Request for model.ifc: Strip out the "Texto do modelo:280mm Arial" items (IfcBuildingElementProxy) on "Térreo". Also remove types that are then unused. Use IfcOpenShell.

First a look at what the model holds.

```python
import ifcopenshell
import ifcopenshell.util.element

model = ifcopenshell.open("model.ifc")
print(model.schema)
storey = next(s for s in model.by_type("IfcBuildingStorey") if s.Name == "Térreo")
proxies = [e for e in ifcopenshell.util.element.get_decomposition(storey) if e.is_a("IfcBuildingElementProxy")]
seen = {}
for e in proxies:
    element_type = ifcopenshell.util.element.get_type(e)
    name = element_type.Name if element_type not in (None, e) else None
    seen[name] = seen.get(name, 0) + 1
for name, count in sorted(seen.items(), key=str):
    print(count, "x", name)
```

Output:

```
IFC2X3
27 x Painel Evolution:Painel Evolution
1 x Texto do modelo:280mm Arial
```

```python
import ifcopenshell
import ifcopenshell.api.root
import ifcopenshell.util.element

model = ifcopenshell.open("model.ifc")

storey = next(s for s in model.by_type("IfcBuildingStorey") if s.Name == "Térreo")
proxies = [e for e in ifcopenshell.util.element.get_decomposition(storey) if e.is_a("IfcBuildingElementProxy")]
targets = [e for e in proxies if (t := ifcopenshell.util.element.get_type(e)) not in (None, e) and t.Name == "Texto do modelo:280mm Arial"]
types = {ifcopenshell.util.element.get_type(e) for e in targets} - {None, *targets}

for e in targets:
    ifcopenshell.api.root.remove_product(model, product=e)
print(len(targets), "removed")

unused = [t for t in types if not ifcopenshell.util.element.get_types(t)]
for t in unused:
    ifcopenshell.api.root.remove_product(model, product=t)
print(len(unused), "unused types removed")

model.write("model_updated.ifc")
```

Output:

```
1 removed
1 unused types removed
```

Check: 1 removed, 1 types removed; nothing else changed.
